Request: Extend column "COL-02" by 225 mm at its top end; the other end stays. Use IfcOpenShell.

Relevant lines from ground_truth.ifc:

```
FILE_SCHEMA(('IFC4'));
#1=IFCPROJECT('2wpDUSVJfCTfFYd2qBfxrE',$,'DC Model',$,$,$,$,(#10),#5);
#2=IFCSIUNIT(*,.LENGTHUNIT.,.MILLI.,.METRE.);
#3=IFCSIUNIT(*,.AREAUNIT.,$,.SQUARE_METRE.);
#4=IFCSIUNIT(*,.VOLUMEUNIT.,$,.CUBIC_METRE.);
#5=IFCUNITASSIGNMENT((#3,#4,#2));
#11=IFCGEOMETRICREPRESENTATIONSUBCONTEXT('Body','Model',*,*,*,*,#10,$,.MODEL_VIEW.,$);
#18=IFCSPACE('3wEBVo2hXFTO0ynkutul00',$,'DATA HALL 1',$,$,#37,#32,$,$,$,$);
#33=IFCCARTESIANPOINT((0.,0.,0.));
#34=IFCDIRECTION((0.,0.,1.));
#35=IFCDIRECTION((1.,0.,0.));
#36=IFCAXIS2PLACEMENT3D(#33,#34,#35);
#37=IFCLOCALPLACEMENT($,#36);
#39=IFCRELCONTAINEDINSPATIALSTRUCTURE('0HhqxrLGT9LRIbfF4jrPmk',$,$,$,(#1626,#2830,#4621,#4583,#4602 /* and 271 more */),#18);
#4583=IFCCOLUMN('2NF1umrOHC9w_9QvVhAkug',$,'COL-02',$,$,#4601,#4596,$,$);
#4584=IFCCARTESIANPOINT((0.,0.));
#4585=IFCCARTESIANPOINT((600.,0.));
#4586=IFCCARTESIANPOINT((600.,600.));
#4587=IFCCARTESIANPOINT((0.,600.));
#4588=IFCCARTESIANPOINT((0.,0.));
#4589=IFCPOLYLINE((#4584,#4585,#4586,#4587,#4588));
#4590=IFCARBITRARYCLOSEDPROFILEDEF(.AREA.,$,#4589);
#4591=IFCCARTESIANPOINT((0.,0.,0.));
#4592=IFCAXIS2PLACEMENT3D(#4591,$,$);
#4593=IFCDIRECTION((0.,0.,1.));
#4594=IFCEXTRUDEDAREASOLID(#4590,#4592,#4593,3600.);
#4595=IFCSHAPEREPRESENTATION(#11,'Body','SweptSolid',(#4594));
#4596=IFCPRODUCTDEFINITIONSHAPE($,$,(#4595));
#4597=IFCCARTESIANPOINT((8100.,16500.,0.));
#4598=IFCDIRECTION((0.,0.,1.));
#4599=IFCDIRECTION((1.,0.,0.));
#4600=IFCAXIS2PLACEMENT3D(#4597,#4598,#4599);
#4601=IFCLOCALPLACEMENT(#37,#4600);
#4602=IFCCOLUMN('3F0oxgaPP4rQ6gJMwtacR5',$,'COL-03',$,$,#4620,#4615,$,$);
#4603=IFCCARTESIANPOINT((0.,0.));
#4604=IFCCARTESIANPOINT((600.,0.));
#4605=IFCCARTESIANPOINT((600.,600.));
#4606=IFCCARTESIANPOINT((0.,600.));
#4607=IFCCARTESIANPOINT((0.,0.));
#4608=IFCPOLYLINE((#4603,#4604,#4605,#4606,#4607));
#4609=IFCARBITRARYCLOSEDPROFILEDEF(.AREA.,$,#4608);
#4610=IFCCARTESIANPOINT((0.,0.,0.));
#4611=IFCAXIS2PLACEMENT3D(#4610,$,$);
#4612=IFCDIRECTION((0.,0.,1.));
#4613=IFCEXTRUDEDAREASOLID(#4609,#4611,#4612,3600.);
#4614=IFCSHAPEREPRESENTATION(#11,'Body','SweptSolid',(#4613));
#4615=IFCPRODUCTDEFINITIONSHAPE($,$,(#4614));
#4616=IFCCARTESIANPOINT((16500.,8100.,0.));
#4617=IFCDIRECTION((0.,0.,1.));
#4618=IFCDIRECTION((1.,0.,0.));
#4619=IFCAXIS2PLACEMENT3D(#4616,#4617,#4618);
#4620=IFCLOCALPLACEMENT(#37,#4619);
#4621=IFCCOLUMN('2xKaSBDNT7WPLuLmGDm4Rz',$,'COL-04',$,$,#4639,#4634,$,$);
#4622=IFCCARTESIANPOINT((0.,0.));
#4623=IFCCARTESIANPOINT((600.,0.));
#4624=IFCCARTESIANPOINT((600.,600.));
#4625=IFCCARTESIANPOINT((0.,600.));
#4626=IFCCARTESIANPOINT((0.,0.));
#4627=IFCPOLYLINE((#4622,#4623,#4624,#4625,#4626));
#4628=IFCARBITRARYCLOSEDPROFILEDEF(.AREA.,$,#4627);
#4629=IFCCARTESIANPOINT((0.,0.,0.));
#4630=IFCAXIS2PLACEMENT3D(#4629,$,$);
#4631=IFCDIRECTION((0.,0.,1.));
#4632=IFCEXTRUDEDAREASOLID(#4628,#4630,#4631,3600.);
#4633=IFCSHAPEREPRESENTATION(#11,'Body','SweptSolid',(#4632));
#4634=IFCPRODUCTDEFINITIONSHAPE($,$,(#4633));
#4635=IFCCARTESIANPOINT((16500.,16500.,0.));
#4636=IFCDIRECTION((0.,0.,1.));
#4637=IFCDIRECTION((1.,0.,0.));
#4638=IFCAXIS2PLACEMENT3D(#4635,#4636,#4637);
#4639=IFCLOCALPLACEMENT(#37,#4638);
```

```python
import ifcopenshell
import ifcopenshell.util.representation
import ifcopenshell.util.unit

model = ifcopenshell.open("ground_truth.ifc")
unit_scale = ifcopenshell.util.unit.calculate_unit_scale(model)

member = model.by_guid("2NF1umrOHC9w_9QvVhAkug")
change = 0.225 / unit_scale

# The extrusion runs towards the end named, so only its depth changes.
body = ifcopenshell.util.representation.get_representation(member, "Model", "Body")
solid = body.Items[0]
old_length = solid.Depth
solid.Depth += change

print(f"length {old_length:g} -> {solid.Depth:g}")

model.write("ground_truth_edited.ifc")
```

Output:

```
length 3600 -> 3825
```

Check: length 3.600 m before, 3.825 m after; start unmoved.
